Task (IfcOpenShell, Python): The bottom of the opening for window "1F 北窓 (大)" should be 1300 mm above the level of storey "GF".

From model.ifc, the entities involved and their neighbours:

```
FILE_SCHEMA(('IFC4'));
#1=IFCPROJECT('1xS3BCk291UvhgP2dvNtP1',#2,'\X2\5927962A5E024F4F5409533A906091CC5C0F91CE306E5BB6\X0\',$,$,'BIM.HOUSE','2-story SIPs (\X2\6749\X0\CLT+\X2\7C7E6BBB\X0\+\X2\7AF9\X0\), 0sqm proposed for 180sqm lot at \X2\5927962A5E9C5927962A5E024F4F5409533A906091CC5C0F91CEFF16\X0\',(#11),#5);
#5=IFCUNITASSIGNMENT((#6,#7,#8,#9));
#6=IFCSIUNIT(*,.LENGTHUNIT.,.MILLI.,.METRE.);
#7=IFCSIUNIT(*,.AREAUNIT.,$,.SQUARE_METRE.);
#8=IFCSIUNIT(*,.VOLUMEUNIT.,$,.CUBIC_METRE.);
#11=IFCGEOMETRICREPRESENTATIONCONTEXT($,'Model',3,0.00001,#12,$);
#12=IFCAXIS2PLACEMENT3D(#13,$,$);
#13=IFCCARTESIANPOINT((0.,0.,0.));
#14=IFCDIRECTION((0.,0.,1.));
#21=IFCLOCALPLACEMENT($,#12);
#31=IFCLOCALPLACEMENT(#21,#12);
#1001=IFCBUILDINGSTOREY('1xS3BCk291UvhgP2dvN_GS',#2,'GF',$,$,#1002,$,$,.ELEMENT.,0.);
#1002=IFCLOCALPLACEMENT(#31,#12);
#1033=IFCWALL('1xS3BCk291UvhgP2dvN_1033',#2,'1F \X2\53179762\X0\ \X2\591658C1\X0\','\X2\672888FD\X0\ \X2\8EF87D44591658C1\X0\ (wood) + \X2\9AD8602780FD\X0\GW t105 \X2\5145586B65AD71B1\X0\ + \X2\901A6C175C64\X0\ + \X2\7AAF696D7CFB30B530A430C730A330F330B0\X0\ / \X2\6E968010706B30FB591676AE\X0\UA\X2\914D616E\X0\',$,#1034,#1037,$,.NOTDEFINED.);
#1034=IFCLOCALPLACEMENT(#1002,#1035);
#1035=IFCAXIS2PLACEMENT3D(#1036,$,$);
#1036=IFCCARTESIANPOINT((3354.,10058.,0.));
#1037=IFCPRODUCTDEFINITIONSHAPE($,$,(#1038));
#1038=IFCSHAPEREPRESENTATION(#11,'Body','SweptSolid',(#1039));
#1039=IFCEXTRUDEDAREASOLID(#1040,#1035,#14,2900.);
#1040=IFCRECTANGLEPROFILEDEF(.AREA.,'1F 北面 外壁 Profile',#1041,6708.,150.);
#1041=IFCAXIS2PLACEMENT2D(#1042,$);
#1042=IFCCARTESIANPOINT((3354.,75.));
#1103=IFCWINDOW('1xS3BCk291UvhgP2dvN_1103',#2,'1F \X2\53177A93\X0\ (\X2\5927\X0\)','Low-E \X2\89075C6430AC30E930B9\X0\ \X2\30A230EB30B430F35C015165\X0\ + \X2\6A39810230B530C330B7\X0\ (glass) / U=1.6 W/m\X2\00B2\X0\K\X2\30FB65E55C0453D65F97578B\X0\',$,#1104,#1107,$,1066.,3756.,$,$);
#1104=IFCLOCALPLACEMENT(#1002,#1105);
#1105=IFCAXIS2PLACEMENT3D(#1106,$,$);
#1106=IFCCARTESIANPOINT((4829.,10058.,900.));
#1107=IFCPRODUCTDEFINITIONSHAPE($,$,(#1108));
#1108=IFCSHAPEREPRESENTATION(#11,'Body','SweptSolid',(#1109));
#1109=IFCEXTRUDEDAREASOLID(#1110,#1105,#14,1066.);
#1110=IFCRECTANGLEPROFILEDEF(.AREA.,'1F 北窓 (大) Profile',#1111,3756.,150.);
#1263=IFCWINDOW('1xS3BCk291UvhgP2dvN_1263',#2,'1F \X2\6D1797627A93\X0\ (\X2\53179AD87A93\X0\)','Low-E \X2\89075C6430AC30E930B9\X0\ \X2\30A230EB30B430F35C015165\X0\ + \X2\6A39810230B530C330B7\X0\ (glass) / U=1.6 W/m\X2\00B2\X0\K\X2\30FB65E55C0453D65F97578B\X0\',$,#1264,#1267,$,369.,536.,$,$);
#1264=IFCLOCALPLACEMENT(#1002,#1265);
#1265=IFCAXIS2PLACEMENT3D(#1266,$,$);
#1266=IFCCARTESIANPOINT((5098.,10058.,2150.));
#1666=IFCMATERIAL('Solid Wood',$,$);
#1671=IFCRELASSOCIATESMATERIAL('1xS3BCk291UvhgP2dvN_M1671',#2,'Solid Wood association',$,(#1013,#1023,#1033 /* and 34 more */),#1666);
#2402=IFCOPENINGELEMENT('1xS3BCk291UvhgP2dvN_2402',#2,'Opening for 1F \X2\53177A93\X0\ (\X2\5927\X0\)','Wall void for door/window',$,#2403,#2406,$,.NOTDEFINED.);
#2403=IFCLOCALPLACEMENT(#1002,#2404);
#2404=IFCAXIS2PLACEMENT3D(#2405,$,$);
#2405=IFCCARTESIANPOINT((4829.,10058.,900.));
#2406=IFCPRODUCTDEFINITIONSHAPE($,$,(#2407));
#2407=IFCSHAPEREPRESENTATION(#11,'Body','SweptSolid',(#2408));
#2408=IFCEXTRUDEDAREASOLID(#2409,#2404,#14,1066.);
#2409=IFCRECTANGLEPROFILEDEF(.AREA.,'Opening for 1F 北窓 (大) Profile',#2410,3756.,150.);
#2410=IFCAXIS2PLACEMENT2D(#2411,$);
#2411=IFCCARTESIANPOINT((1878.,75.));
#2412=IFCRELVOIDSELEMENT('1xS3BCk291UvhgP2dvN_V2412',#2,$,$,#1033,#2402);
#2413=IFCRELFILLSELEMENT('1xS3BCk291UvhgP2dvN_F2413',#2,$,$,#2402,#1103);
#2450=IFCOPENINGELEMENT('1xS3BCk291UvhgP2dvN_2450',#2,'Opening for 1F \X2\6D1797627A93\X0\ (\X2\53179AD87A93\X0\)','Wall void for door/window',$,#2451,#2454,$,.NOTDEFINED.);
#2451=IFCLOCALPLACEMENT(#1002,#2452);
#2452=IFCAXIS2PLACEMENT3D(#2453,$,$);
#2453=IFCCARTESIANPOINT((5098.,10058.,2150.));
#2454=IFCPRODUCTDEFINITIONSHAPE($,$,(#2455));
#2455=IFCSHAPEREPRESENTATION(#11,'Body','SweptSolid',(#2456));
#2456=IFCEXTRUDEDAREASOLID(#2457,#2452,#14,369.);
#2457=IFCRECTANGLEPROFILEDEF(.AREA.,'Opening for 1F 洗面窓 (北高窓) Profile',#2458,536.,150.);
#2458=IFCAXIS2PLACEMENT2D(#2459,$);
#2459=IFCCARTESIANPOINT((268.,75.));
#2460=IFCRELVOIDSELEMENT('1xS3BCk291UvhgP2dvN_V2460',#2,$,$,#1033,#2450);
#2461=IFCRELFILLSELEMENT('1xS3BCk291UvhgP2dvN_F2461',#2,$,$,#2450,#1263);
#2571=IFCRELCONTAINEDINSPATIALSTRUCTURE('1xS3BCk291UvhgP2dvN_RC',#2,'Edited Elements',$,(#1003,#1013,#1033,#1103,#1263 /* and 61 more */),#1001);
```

```python
import numpy as np
import ifcopenshell
import ifcopenshell.api.geometry
import ifcopenshell.geom
import ifcopenshell.util.element
import ifcopenshell.util.placement
import ifcopenshell.util.shape
import ifcopenshell.util.unit

model = ifcopenshell.open("model.ifc")
unit_scale = ifcopenshell.util.unit.calculate_unit_scale(model)

window = model.by_id(1103)
opening = window.FillsVoids[0].RelatingOpeningElement
storey = ifcopenshell.util.element.get_container(window, ifc_class="IfcBuildingStorey")
level = ifcopenshell.util.placement.get_local_placement(storey.ObjectPlacement)[2, 3]

# The opening's origin need not be at the sill, so measure its lowest point.
shape = ifcopenshell.geom.create_shape(ifcopenshell.geom.settings(), opening)
bottom = ifcopenshell.util.shape.get_shape_bottom_elevation(shape, shape.geometry) / unit_scale
dz = level + 1.3 / unit_scale - bottom

shift = np.array([0.0, 0.0, dz])
# The window is not placed relative to its opening, so move both.
for product in (opening, window):
    matrix = ifcopenshell.util.placement.get_local_placement(product.ObjectPlacement)
    matrix[:3, 3] += shift
    ifcopenshell.api.geometry.edit_object_placement(model, product=product, matrix=matrix, is_si=False)

print(f"moved by {dz * unit_scale:+.3f} m")

model.write("model_rev.ifc")
```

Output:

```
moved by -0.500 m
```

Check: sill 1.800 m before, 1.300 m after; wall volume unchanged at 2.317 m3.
